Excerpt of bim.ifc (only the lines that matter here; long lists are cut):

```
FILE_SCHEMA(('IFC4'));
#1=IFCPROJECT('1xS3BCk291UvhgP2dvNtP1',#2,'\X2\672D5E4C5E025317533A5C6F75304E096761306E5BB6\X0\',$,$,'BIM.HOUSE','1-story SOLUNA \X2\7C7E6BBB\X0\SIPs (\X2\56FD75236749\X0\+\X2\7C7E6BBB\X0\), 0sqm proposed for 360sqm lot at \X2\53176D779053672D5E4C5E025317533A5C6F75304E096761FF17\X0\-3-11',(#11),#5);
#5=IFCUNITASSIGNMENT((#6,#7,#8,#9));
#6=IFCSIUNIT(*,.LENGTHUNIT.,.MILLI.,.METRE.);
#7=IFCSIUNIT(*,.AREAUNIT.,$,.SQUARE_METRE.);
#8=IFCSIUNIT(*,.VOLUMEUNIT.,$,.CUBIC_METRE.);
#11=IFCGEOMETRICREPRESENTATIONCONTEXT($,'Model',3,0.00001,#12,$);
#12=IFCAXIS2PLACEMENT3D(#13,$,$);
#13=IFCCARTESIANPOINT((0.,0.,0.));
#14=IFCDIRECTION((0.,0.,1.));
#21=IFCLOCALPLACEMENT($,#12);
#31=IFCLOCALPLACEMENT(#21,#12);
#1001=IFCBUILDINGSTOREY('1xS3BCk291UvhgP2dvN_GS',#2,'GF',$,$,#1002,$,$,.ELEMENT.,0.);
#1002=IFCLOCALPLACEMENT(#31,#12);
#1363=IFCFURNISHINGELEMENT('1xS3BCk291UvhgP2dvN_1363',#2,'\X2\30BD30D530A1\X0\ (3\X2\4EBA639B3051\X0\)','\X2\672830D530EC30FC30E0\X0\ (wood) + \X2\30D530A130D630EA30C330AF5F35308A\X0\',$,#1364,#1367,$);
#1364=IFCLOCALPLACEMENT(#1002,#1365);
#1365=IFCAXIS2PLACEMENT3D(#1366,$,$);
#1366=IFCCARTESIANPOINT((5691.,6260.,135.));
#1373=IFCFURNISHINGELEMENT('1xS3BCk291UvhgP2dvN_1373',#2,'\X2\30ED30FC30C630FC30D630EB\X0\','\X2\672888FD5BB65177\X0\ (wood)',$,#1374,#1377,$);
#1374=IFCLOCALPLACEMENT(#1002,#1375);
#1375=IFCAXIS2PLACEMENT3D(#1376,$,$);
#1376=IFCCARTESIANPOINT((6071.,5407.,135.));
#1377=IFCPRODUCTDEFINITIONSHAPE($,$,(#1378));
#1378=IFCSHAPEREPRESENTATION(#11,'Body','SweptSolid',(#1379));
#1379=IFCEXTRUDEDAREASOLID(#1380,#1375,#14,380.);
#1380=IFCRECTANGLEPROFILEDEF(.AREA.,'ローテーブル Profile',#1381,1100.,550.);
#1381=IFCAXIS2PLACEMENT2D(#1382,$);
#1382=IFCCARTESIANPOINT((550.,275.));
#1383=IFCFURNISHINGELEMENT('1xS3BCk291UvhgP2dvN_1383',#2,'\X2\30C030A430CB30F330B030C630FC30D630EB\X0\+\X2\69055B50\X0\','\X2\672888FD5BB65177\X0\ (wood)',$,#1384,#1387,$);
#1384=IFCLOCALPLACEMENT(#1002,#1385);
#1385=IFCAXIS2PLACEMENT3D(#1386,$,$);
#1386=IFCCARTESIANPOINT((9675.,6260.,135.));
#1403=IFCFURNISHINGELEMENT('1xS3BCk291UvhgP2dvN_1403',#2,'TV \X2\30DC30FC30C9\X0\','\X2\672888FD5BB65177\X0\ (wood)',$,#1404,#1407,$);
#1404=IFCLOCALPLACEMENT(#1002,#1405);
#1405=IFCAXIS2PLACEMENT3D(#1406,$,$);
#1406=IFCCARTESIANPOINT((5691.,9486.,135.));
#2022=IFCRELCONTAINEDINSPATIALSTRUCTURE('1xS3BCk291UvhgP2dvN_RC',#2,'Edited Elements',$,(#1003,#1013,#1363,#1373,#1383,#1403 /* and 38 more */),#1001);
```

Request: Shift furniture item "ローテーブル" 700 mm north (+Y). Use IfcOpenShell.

```python
import ifcopenshell
import ifcopenshell.api.geometry
import ifcopenshell.util.placement
import ifcopenshell.util.unit

model = ifcopenshell.open("bim.ifc")
unit_scale = ifcopenshell.util.unit.calculate_unit_scale(model)

item = model.by_guid("1xS3BCk291UvhgP2dvN_1373")
matrix = ifcopenshell.util.placement.get_local_placement(item.ObjectPlacement)
matrix[1, 3] += 0.7 / unit_scale
ifcopenshell.api.geometry.edit_object_placement(model, product=item, matrix=matrix, is_si=False)

print(ifcopenshell.util.placement.get_local_placement(item.ObjectPlacement).round(3) + 0.0)

model.write("bim_rev.ifc")
```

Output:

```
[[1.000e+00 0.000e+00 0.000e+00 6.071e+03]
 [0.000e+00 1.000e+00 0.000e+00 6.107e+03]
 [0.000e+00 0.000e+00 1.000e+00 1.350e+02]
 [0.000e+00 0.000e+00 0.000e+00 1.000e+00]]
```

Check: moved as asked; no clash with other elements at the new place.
